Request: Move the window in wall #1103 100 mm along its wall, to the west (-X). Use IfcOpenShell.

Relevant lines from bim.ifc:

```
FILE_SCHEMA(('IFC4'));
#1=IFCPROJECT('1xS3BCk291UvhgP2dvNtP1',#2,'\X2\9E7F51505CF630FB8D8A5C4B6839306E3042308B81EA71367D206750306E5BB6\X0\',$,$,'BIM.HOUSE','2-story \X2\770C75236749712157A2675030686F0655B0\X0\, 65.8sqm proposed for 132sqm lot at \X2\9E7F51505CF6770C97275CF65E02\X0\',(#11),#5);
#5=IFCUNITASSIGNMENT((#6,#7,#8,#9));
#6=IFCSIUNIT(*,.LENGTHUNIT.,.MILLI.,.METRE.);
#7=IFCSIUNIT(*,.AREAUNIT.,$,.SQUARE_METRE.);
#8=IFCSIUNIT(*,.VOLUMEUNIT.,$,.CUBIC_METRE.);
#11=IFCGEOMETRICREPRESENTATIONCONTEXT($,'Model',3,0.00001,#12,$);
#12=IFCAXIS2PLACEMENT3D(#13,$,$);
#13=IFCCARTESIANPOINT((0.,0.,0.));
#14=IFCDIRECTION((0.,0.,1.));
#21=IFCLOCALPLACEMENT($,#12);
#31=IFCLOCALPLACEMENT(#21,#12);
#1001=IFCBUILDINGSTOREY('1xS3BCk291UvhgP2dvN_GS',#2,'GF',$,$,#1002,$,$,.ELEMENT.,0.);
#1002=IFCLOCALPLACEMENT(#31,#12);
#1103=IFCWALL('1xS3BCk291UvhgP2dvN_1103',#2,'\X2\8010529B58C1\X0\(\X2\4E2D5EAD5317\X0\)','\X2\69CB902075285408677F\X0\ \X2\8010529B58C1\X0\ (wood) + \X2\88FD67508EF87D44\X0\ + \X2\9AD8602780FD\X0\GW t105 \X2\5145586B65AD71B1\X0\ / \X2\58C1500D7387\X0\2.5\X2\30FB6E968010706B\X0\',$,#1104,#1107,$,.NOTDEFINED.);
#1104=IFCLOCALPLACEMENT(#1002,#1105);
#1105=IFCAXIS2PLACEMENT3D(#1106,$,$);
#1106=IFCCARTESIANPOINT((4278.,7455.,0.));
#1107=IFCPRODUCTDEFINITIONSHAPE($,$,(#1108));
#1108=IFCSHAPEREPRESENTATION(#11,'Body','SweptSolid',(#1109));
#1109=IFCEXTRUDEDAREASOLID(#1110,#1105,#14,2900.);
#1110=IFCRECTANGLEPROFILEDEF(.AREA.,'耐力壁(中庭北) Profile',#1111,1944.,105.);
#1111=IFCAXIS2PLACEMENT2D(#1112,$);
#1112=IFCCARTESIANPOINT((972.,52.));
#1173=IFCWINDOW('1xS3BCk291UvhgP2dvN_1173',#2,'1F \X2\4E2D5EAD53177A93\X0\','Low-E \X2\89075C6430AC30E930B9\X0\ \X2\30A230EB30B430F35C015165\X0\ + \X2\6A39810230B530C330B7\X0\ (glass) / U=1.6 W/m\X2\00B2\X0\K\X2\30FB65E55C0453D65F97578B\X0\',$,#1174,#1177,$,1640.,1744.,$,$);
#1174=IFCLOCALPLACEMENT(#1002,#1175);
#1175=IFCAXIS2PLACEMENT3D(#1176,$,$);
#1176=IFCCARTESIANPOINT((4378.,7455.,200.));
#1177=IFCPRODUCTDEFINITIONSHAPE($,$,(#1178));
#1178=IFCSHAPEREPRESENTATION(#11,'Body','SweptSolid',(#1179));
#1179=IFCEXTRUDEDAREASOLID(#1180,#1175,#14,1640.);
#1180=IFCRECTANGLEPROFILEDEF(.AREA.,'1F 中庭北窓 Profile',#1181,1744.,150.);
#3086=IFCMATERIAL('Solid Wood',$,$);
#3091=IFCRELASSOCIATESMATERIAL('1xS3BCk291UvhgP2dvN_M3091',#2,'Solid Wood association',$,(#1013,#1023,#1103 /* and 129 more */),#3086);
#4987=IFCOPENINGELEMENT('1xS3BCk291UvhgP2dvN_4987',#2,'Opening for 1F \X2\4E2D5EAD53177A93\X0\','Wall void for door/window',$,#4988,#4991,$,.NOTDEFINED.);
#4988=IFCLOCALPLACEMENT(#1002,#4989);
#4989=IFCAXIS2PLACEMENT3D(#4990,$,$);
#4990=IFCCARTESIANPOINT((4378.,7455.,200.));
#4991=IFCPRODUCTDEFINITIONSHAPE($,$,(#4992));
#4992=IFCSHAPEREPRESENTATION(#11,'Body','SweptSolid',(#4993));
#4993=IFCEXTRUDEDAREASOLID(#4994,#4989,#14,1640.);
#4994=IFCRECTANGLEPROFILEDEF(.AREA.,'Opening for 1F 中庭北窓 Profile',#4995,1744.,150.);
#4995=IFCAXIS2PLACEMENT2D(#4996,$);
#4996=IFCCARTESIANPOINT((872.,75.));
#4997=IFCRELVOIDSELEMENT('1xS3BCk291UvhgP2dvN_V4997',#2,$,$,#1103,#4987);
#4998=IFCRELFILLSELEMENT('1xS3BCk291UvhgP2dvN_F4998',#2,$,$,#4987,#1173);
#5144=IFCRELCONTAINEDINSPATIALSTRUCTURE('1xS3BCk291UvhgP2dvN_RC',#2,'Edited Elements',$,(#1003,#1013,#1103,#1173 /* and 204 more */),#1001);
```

```python
import ifcopenshell
import ifcopenshell.api.geometry
import ifcopenshell.util.placement
import ifcopenshell.util.unit

model = ifcopenshell.open("bim.ifc")
unit_scale = ifcopenshell.util.unit.calculate_unit_scale(model)

window = model.by_id(1173)
opening = window.FillsVoids[0].RelatingOpeningElement
wall = opening.VoidsElements[0].RelatingBuildingElement

wall_matrix = ifcopenshell.util.placement.get_local_placement(wall.ObjectPlacement)
shift = wall_matrix[:3, 0] * -0.1 / unit_scale
before = ifcopenshell.util.placement.get_local_placement(window.ObjectPlacement)[:3, 3].copy()

# The window is not placed relative to its opening, so move both.
for product in (opening, window):
    matrix = ifcopenshell.util.placement.get_local_placement(product.ObjectPlacement)
    matrix[:3, 3] += shift
    ifcopenshell.api.geometry.edit_object_placement(model, product=product, matrix=matrix, is_si=False)

after = ifcopenshell.util.placement.get_local_placement(window.ObjectPlacement)[:3, 3]
print("window moved by", (after - before).round(3) + 0.0)

model.write("bim_updated.ifc")
```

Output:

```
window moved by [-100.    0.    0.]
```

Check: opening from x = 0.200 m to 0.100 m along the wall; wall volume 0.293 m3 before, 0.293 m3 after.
